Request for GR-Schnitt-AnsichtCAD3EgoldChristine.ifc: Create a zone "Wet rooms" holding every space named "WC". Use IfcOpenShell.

First a look at what the model holds.

```python
import ifcopenshell

model = ifcopenshell.open("GR-Schnitt-AnsichtCAD3EgoldChristine.ifc")
print(model.schema)
seen = {}
for space in model.by_type("IfcSpace"):
    seen[space.LongName] = seen.get(space.LongName, 0) + 1
for name, count in sorted(seen.items(), key=str):
    print(count, "x", name)
print("zones:", [z.Name for z in model.by_type("IfcZone")][:20])
```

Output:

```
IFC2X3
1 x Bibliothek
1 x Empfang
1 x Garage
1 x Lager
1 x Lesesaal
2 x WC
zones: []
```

```python
import ifcopenshell
import ifcopenshell.api.group
import ifcopenshell.api.root

model = ifcopenshell.open("GR-Schnitt-AnsichtCAD3EgoldChristine.ifc")

names = {"WC"}
spaces = [s for s in model.by_type("IfcSpace") if s.LongName in names]

zone = ifcopenshell.api.root.create_entity(model, ifc_class="IfcZone", name="Wet rooms")
ifcopenshell.api.group.assign_group(model, products=spaces, group=zone)
print(len(spaces), "spaces in", zone.Name)

model.write("GR-Schnitt-AnsichtCAD3EgoldChristine-out.ifc")
```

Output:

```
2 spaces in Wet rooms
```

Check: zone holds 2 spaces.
